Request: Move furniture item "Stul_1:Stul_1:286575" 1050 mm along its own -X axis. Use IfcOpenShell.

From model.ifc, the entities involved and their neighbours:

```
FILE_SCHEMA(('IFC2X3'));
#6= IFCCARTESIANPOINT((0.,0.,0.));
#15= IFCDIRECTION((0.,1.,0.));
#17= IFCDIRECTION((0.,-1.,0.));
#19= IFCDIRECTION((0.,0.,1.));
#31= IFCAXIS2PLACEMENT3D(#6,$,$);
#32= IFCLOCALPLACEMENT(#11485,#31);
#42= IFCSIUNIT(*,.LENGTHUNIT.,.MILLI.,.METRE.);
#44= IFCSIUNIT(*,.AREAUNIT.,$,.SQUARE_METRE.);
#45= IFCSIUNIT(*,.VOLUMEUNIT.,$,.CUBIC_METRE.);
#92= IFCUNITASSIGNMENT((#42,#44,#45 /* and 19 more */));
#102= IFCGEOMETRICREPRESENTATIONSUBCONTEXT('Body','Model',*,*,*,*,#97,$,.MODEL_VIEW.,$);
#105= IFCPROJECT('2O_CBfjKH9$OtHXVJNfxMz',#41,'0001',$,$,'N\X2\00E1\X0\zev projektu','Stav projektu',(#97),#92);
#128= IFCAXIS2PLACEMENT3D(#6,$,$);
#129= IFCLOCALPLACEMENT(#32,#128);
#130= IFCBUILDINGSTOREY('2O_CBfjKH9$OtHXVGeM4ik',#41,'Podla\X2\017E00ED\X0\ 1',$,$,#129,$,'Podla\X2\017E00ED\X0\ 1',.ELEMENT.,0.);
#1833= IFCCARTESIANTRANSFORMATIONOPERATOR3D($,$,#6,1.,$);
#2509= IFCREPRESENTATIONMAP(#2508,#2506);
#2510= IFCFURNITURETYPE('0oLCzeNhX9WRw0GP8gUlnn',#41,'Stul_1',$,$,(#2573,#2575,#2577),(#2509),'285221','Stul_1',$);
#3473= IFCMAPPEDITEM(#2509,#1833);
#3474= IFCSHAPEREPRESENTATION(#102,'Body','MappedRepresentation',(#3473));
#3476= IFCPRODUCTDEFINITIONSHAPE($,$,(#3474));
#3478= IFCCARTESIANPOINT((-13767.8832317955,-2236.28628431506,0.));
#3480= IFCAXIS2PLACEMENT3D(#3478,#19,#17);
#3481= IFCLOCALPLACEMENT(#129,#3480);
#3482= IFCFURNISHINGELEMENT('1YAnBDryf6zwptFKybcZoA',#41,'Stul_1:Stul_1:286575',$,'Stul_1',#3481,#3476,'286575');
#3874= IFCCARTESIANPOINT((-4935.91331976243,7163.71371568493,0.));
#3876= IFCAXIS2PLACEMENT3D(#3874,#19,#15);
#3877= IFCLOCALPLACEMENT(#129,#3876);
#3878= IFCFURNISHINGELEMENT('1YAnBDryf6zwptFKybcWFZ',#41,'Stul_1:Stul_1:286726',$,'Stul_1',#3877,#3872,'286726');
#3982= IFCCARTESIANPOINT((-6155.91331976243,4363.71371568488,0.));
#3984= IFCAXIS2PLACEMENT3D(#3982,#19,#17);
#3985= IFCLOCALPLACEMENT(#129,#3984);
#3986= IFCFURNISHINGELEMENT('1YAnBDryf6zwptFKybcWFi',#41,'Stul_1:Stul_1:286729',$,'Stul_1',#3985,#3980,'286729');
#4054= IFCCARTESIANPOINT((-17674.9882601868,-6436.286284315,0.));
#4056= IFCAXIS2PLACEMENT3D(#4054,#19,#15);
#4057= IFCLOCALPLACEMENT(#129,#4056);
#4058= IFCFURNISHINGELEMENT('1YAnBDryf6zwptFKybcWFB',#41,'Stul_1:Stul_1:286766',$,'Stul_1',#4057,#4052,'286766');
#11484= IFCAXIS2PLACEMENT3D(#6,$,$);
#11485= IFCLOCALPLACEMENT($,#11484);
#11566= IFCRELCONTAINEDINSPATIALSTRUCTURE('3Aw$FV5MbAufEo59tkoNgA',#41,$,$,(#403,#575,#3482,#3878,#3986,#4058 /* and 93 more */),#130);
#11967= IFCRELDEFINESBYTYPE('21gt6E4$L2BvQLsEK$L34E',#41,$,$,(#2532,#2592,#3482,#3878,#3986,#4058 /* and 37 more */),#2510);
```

```python
import ifcopenshell
import ifcopenshell.api.geometry
import ifcopenshell.util.placement
import ifcopenshell.util.unit

model = ifcopenshell.open("model.ifc")
unit_scale = ifcopenshell.util.unit.calculate_unit_scale(model)

item = model.by_id(3482)
matrix = ifcopenshell.util.placement.get_local_placement(item.ObjectPlacement)
matrix[:3, 3] -= matrix[:3, 0] * 1.05 / unit_scale
ifcopenshell.api.geometry.edit_object_placement(model, product=item, matrix=matrix, is_si=False)

print(ifcopenshell.util.placement.get_local_placement(item.ObjectPlacement).round(3) + 0.0)

model.write("model_v2.ifc")
```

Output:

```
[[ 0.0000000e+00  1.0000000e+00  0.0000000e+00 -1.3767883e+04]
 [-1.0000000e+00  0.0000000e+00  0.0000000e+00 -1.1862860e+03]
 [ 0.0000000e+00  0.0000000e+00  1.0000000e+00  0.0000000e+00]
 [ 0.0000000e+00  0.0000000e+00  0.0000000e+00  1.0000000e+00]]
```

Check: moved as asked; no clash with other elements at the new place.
